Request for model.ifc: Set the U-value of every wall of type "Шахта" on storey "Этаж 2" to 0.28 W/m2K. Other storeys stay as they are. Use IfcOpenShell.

First a look at what the model holds.

```python
import ifcopenshell
import ifcopenshell.util.element

model = ifcopenshell.open("model.ifc")
print(model.schema)
storey = next(s for s in model.by_type("IfcBuildingStorey") if s.Name == "Этаж 2")
walls = [e for e in ifcopenshell.util.element.get_decomposition(storey) if e.is_a("IfcWall")]
seen = {}
for e in walls:
    element_type = ifcopenshell.util.element.get_type(e)
    key = (element_type.Name if element_type != e and element_type else None, ifcopenshell.util.element.get_pset(e, "Pset_WallCommon", "ThermalTransmittance"))
    seen[key] = seen.get(key, 0) + 1
for (name, value), count in sorted(seen.items(), key=str):
    print(count, "x", name, "|", value)
```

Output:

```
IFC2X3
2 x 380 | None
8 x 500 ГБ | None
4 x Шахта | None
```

```python
import ifcopenshell
import ifcopenshell.api.pset
import ifcopenshell.util.element

model = ifcopenshell.open("model.ifc")

storey = next(s for s in model.by_type("IfcBuildingStorey") if s.Name == "Этаж 2")
walls = [e for e in ifcopenshell.util.element.get_decomposition(storey) if e.is_a("IfcWall")]

count = 0
for e in walls:
    element_type = ifcopenshell.util.element.get_type(e)
    if element_type in (None, e) or element_type.Name != "Шахта":
        continue
    # add_pset returns the element's existing set when there is one.
    pset = ifcopenshell.api.pset.add_pset(model, product=e, name="Pset_WallCommon")
    ifcopenshell.api.pset.edit_pset(model, pset=pset, properties={"ThermalTransmittance": 0.28})
    count += 1

print(count, "walls updated")

model.write("model_edited.ifc")
```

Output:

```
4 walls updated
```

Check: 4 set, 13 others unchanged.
